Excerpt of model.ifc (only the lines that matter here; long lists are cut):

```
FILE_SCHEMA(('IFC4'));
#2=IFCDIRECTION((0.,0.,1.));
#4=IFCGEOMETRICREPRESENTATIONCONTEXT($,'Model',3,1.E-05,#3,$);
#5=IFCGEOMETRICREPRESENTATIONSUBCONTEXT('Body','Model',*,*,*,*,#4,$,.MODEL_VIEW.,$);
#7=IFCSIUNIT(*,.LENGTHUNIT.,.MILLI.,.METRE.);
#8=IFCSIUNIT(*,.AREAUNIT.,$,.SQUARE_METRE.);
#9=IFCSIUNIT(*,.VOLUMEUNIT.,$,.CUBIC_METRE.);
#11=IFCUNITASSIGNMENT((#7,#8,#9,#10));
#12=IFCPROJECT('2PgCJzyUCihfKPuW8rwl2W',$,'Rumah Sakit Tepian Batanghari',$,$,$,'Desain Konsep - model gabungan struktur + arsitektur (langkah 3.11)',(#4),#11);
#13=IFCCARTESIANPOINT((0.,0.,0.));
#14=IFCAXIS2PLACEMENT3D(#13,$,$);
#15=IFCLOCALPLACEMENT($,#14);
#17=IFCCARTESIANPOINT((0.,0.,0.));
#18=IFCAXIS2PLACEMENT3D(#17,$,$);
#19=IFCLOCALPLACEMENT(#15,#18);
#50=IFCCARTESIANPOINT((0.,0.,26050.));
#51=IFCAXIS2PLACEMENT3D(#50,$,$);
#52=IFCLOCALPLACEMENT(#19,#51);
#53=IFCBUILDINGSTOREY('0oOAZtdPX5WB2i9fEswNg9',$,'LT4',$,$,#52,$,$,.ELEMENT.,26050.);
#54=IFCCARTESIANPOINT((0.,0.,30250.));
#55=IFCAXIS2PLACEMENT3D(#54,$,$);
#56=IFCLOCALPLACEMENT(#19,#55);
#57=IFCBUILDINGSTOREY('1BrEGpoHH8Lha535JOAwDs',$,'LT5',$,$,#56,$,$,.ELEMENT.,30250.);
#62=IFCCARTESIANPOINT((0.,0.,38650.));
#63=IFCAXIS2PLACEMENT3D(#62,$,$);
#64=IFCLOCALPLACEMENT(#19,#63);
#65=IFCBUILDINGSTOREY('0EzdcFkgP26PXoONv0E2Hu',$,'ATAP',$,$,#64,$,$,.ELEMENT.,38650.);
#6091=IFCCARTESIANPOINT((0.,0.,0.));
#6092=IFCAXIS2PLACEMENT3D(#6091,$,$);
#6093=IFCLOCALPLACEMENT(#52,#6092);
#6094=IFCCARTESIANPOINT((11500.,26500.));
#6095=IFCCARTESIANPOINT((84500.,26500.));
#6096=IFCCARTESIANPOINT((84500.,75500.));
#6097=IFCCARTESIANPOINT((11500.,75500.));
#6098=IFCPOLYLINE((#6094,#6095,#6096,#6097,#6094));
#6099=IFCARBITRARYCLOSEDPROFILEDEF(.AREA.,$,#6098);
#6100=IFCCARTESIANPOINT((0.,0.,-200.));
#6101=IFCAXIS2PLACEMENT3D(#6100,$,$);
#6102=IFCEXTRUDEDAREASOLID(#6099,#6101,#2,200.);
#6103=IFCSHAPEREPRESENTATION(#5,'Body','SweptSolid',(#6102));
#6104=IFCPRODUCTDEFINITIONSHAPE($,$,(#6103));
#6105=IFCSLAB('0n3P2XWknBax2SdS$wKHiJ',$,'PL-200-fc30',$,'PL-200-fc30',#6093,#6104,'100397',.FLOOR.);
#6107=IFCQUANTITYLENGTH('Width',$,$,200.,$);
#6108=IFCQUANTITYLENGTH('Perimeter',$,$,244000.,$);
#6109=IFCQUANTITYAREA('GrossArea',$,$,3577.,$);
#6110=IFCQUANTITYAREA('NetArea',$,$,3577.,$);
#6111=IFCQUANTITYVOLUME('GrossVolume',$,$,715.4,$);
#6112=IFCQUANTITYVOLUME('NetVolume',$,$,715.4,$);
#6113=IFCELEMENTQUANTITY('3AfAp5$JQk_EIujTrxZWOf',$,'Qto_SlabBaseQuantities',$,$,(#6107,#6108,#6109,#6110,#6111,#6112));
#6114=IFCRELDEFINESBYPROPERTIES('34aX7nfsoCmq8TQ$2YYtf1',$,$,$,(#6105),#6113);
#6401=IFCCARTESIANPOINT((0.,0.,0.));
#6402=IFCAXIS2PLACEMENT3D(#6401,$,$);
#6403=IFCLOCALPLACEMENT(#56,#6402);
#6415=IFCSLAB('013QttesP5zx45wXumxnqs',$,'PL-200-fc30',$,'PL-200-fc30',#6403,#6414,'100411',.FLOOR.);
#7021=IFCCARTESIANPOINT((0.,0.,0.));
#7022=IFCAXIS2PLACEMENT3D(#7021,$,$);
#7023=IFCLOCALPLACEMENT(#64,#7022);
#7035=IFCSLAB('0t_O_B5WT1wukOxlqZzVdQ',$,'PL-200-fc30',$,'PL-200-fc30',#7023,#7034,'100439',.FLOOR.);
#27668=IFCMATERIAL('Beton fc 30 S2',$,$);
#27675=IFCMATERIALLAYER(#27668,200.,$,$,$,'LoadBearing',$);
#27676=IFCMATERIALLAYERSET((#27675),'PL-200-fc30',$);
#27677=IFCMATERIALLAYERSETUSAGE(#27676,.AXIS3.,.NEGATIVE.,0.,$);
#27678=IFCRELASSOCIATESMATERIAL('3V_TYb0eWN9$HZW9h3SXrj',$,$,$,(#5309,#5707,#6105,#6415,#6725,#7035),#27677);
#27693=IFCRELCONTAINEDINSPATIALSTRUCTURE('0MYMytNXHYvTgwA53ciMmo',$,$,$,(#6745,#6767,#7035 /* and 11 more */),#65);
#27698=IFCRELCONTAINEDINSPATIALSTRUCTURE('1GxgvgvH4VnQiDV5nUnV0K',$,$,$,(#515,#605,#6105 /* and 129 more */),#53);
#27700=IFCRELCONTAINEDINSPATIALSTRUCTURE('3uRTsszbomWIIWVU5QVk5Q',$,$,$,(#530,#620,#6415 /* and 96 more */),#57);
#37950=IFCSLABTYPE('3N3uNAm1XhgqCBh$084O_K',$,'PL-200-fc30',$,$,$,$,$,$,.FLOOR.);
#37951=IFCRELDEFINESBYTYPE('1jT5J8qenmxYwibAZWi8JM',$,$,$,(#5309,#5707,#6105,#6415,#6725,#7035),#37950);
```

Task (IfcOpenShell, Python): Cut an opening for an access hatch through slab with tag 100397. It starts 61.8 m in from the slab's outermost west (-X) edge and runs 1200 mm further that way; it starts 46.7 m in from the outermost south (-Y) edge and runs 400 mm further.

```python
import numpy as np
import ifcopenshell
import ifcopenshell.api.feature
import ifcopenshell.api.geometry
import ifcopenshell.api.pset
import ifcopenshell.api.root
import ifcopenshell.geom
import ifcopenshell.util.element
import ifcopenshell.util.placement
import ifcopenshell.util.representation
import ifcopenshell.util.shape
import ifcopenshell.util.unit

model = ifcopenshell.open("model.ifc")
unit_scale = ifcopenshell.util.unit.calculate_unit_scale(model)
area_scale = ifcopenshell.util.unit.calculate_unit_scale(model, "AREAUNIT")
volume_scale = ifcopenshell.util.unit.calculate_unit_scale(model, "VOLUMEUNIT")
settings = ifcopenshell.geom.settings()


def volume(element):
    """Net volume in cubic metres, openings subtracted."""
    shape = ifcopenshell.geom.create_shape(settings, element)
    return ifcopenshell.util.shape.get_volume(shape.geometry)


slab = model.by_guid("0n3P2XWknBax2SdS$wKHiJ")
before = volume(slab)

# Extent in the slab's own axes, in metres. The edges named are its -X and -Y sides.
slab_shape = ifcopenshell.geom.create_shape(settings, slab)
vertices = ifcopenshell.util.shape.get_vertices(slab_shape.geometry)
x_min, y_min, bottom = vertices.min(axis=0)
top = vertices[:, 2].max()

opening = ifcopenshell.api.root.create_entity(model, ifc_class="IfcOpeningElement", name="Access hatch opening", predefined_type="OPENING")
context = ifcopenshell.util.representation.get_context(model, "Model", "Body", "MODEL_VIEW")
width, depth = 1.2, 0.4
outline = [(0.0, 0.0), (width, 0.0), (width, depth), (0.0, depth), (0.0, 0.0)]
# Overshoot both faces by 50 mm so the cut is clean.
shape = ifcopenshell.api.geometry.add_slab_representation(
    model, context=context, depth=top - bottom + 0.1, polyline=outline
)
ifcopenshell.api.geometry.assign_representation(model, product=opening, representation=shape)

matrix = ifcopenshell.util.placement.get_local_placement(slab.ObjectPlacement)
matrix[:, 3] = matrix @ np.append(np.array([x_min + 61.8, y_min + 46.7, bottom - 0.05]) / unit_scale, 1.0)
ifcopenshell.api.geometry.edit_object_placement(model, product=opening, matrix=matrix, is_si=False)
ifcopenshell.api.feature.add_feature(model, feature=opening, element=slab)

after = volume(slab)

# Update the slab's stored quantities.
qto = model.by_id(ifcopenshell.util.element.get_pset(slab, "Qto_SlabBaseQuantities", should_inherit=False)["id"])
ifcopenshell.api.pset.edit_qto(model, qto=qto, properties={
    "NetArea": after / (top - bottom) / area_scale,
    "NetVolume": after / volume_scale,
})

print(f"slab volume {before:.3f} -> {after:.3f} m3")

model.write("model_rev.ifc")
```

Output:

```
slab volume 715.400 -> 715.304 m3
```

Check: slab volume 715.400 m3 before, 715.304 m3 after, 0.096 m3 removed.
